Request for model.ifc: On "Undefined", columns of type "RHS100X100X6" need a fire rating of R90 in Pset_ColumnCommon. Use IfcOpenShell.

First a look at what the model holds.

```python
import ifcopenshell
import ifcopenshell.util.element

model = ifcopenshell.open("model.ifc")
print(model.schema)
storey = next(s for s in model.by_type("IfcBuildingStorey") if s.Name == "Undefined")
columns = [e for e in ifcopenshell.util.element.get_decomposition(storey) if e.is_a("IfcColumn")]
seen = {}
for e in columns:
    element_type = ifcopenshell.util.element.get_type(e)
    key = (element_type.Name if element_type != e and element_type else None, ifcopenshell.util.element.get_pset(e, "Pset_ColumnCommon", "FireRating"))
    seen[key] = seen.get(key, 0) + 1
for (name, value), count in sorted(seen.items(), key=str):
    print(count, "x", name, "|", value)
```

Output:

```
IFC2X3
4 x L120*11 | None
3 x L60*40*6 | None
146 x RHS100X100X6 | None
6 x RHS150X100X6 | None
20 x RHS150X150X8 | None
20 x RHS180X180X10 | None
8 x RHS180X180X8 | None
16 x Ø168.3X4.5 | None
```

```python
import ifcopenshell
import ifcopenshell.api.pset
import ifcopenshell.util.element

model = ifcopenshell.open("model.ifc")

storey = next(s for s in model.by_type("IfcBuildingStorey") if s.Name == "Undefined")
columns = [e for e in ifcopenshell.util.element.get_decomposition(storey) if e.is_a("IfcColumn")]

count = 0
for e in columns:
    element_type = ifcopenshell.util.element.get_type(e)
    if element_type in (None, e) or element_type.Name != "RHS100X100X6":
        continue
    found = ifcopenshell.util.element.get_pset(e, "Pset_ColumnCommon", should_inherit=False)
    if found:
        pset = model.by_id(found["id"])
        if len(ifcopenshell.util.element.get_elements_by_pset(pset)) > 1:
            pset = ifcopenshell.api.pset.unshare_pset(model, products=[e], pset=pset)[0]
    else:
        pset = ifcopenshell.api.pset.add_pset(model, product=e, name="Pset_ColumnCommon")
    ifcopenshell.api.pset.edit_pset(model, pset=pset, properties={"FireRating": "R90"})
    count += 1

print(count, "columns updated")

model.write("model_v2.ifc")
```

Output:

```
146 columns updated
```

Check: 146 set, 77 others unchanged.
